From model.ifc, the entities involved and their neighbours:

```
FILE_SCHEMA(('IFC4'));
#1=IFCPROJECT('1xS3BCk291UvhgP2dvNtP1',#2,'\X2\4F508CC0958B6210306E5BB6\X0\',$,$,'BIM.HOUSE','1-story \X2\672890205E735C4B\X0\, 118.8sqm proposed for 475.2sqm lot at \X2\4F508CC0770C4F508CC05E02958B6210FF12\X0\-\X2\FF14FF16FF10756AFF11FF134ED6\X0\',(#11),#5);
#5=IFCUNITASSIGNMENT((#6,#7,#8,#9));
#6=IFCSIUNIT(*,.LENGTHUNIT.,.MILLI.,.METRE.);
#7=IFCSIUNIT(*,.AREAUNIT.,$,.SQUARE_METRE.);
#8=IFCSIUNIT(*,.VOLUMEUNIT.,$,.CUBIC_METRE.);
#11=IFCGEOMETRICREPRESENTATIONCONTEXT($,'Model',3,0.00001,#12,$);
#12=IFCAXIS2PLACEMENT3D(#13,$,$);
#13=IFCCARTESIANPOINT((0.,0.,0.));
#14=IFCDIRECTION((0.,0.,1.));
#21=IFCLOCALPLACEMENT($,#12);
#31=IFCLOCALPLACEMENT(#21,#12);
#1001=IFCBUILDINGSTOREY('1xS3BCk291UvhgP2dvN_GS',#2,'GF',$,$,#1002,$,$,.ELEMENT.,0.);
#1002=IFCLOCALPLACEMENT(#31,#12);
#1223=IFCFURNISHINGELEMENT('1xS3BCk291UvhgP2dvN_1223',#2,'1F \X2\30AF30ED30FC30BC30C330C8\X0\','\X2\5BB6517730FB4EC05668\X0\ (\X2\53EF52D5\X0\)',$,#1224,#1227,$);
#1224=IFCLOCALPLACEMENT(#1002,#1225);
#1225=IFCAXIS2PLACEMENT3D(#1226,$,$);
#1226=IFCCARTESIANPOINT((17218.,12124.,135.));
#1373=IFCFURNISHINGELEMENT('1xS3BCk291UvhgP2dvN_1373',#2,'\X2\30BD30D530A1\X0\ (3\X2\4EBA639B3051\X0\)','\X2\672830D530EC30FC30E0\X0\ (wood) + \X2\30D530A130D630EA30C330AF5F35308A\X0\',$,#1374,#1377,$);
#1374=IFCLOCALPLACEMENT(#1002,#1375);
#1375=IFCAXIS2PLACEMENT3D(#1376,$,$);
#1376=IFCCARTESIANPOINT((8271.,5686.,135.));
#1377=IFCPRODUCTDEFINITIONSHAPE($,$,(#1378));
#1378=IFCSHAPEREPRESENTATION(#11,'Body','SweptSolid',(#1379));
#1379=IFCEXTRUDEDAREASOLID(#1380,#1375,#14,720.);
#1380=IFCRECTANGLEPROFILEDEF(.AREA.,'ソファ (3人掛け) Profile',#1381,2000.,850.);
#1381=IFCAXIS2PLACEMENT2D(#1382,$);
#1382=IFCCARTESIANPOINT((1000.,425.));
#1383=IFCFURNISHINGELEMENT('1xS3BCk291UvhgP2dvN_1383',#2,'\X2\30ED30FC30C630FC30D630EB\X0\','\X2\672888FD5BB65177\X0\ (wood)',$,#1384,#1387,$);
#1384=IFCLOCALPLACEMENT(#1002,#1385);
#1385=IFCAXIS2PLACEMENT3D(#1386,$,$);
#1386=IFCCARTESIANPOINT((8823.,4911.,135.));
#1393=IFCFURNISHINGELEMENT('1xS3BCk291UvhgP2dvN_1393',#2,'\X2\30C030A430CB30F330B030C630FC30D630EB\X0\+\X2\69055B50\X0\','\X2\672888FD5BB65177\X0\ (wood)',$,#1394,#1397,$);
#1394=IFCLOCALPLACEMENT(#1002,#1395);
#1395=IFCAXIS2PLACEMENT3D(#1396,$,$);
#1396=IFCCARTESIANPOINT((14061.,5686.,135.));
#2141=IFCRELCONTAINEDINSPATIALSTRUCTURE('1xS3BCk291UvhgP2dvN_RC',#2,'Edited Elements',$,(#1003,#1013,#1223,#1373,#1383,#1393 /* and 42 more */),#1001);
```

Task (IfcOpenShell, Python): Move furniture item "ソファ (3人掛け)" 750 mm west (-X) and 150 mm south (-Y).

```python
import ifcopenshell
import ifcopenshell.api.geometry
import ifcopenshell.util.placement
import ifcopenshell.util.unit

model = ifcopenshell.open("model.ifc")
unit_scale = ifcopenshell.util.unit.calculate_unit_scale(model)

item = model.by_guid("1xS3BCk291UvhgP2dvN_1373")
matrix = ifcopenshell.util.placement.get_local_placement(item.ObjectPlacement)
matrix[0, 3] -= 0.75 / unit_scale
matrix[1, 3] -= 0.15 / unit_scale
ifcopenshell.api.geometry.edit_object_placement(model, product=item, matrix=matrix, is_si=False)

print(ifcopenshell.util.placement.get_local_placement(item.ObjectPlacement).round(3) + 0.0)

model.write("model_rev.ifc")
```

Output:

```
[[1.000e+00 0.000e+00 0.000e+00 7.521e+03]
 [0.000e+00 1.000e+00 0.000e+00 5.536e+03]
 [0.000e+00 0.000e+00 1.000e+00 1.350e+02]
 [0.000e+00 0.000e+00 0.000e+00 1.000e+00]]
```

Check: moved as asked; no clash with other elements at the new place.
